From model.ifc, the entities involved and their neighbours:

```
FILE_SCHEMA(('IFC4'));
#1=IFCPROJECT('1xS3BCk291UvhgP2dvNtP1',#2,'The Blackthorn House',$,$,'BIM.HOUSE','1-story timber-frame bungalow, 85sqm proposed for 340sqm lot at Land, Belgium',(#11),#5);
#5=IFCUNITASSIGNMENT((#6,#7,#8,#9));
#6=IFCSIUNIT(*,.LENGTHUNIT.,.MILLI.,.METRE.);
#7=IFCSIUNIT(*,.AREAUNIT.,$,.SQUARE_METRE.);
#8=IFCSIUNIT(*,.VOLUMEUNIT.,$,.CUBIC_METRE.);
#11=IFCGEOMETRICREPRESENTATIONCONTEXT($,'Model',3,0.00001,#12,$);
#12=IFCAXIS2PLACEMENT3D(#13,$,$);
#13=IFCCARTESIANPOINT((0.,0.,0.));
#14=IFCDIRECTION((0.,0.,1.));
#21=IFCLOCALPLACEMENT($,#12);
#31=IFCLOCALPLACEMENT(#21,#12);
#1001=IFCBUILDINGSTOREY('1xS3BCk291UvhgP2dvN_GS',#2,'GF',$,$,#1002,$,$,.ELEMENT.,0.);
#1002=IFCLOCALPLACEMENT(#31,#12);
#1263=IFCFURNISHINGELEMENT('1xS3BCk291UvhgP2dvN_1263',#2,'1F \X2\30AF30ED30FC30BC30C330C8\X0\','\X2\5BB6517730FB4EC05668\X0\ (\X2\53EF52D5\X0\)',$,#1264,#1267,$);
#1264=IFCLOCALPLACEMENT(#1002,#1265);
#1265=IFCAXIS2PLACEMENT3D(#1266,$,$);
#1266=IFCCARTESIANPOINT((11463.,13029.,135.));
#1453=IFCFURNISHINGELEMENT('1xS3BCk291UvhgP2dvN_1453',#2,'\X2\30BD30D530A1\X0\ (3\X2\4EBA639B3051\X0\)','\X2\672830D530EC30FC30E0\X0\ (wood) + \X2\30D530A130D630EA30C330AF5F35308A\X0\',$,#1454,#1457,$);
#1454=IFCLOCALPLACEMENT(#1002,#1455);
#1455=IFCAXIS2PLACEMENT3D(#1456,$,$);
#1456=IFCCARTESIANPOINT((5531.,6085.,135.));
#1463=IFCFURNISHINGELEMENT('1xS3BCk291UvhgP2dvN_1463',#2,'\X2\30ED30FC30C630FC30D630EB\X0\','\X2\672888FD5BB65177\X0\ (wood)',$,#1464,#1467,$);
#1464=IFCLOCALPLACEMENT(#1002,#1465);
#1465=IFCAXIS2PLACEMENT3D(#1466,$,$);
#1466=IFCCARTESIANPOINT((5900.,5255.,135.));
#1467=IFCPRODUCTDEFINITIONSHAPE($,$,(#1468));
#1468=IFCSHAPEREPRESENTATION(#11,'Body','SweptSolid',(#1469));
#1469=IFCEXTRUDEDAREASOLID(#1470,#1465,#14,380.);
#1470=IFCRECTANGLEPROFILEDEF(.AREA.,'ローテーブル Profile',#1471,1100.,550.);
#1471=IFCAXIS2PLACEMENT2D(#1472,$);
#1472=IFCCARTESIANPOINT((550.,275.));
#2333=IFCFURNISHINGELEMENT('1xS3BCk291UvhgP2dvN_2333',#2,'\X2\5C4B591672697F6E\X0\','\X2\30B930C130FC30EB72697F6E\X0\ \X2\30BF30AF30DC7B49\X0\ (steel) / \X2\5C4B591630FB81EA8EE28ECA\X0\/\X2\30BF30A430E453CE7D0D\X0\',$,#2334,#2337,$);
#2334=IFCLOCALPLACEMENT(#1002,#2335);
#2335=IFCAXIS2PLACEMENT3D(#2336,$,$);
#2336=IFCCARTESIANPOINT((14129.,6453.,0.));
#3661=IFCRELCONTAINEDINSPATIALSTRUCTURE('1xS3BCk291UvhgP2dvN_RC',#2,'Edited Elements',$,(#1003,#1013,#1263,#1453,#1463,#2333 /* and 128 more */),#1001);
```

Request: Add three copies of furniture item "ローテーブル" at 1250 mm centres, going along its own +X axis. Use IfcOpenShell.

```python
import ifcopenshell
import ifcopenshell.api.geometry
import ifcopenshell.api.root
import ifcopenshell.util.element
import ifcopenshell.util.placement
import ifcopenshell.util.unit

model = ifcopenshell.open("model.ifc")
unit_scale = ifcopenshell.util.unit.calculate_unit_scale(model)


def reuse_history(source, copy):
    """copy_class also copies each property set's owner history, people and application; keep the originals."""
    for rel in copy.IsDefinedBy:
        if rel.is_a("IfcRelDefinesByProperties") and (history := rel.RelatingPropertyDefinition.OwnerHistory):
            rel.RelatingPropertyDefinition.OwnerHistory = source.OwnerHistory
            ifcopenshell.util.element.remove_deep2(model, history)


source = model.by_guid("1xS3BCk291UvhgP2dvN_1463")
base = ifcopenshell.util.placement.get_local_placement(source.ObjectPlacement)
step = base[:3, 0] * 1.25 / unit_scale

for i in range(1, 4):
    copy = ifcopenshell.api.root.copy_class(model, product=source)
    copy.Representation = ifcopenshell.util.element.copy_deep(
        model, source.Representation, exclude=["IfcGeometricRepresentationContext", "IfcRepresentationMap"]
    )
    reuse_history(source, copy)
    matrix = base.copy()
    matrix[:3, 3] += i * step
    print("added at", matrix[:3, 3].round(3) + 0.0)
    ifcopenshell.api.geometry.edit_object_placement(model, product=copy, matrix=matrix, is_si=False)

model.write("model_updated.ifc")
```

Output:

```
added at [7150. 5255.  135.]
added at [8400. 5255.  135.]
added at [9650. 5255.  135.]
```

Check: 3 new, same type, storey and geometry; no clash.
